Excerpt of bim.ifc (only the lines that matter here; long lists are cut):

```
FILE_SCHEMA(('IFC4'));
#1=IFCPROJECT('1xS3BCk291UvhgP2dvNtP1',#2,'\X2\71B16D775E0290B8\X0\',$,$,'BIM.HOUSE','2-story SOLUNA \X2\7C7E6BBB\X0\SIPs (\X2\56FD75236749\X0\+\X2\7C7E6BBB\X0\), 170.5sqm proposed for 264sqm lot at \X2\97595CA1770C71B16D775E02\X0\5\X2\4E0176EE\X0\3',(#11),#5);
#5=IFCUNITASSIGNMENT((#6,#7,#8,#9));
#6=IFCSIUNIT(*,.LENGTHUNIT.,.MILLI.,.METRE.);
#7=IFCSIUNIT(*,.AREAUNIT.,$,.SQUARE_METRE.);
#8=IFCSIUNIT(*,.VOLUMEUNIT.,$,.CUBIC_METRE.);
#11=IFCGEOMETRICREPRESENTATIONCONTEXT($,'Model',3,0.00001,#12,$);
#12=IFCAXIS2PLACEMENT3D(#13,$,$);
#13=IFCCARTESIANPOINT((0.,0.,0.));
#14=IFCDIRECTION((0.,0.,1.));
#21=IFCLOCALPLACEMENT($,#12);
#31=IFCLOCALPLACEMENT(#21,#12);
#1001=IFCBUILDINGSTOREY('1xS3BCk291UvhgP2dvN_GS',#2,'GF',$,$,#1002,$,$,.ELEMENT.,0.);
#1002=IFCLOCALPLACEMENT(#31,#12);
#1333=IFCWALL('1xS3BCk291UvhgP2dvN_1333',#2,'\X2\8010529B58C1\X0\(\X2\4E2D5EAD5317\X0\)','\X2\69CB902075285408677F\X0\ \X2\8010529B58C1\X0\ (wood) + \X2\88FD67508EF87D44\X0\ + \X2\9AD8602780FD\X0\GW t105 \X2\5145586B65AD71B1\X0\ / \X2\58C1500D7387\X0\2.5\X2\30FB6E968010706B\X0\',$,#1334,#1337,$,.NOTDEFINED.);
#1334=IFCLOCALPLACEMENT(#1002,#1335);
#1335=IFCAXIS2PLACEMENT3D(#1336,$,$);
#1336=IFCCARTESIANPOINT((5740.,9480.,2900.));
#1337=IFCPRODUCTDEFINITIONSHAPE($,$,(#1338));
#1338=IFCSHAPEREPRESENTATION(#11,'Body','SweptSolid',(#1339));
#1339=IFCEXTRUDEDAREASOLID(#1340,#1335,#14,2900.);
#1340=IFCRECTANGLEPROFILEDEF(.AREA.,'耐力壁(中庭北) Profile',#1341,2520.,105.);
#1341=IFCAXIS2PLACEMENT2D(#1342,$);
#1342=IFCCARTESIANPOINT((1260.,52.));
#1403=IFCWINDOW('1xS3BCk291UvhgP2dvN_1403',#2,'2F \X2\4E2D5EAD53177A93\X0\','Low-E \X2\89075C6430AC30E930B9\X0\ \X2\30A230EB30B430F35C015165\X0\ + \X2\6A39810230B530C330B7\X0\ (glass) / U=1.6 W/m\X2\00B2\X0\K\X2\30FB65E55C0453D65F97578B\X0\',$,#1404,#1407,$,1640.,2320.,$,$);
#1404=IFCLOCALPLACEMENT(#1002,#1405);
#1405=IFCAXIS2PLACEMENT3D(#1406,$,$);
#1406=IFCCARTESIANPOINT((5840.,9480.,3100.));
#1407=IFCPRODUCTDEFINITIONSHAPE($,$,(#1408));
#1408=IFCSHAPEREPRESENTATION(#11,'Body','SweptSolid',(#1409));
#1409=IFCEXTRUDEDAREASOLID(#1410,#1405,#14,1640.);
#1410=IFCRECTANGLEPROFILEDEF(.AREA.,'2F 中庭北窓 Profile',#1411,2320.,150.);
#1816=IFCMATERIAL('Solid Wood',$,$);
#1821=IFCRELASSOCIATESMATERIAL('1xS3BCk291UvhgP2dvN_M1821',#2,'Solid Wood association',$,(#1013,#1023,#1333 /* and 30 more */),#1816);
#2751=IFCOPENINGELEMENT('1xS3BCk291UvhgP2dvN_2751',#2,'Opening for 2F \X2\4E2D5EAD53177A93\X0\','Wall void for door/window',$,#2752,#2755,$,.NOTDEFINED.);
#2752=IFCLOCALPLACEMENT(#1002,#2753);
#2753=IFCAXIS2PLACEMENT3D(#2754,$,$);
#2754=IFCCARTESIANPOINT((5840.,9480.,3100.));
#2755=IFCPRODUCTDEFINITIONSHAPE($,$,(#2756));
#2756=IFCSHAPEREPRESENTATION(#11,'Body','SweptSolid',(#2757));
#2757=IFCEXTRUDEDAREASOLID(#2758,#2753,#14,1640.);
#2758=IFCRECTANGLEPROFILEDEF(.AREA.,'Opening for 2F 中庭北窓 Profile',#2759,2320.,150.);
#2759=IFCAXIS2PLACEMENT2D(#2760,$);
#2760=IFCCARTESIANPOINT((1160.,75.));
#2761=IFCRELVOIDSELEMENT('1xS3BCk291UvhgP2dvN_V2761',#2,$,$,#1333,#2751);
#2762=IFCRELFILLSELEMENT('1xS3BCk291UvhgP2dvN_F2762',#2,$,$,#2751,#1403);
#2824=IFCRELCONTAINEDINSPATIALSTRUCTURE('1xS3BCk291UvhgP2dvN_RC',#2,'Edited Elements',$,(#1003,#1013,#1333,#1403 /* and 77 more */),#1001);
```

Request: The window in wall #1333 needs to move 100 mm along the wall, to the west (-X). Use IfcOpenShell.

```python
import ifcopenshell
import ifcopenshell.api.geometry
import ifcopenshell.util.placement

model = ifcopenshell.open("bim.ifc")

window = model.by_guid("1xS3BCk291UvhgP2dvN_1403")
opening = window.FillsVoids[0].RelatingOpeningElement
wall = opening.VoidsElements[0].RelatingBuildingElement

wall_matrix = ifcopenshell.util.placement.get_local_placement(wall.ObjectPlacement)
shift = wall_matrix[:3, 0] * -100.0
before = ifcopenshell.util.placement.get_local_placement(window.ObjectPlacement)[:3, 3].copy()

# The window is not placed relative to its opening, so move both.
for product in (opening, window):
    matrix = ifcopenshell.util.placement.get_local_placement(product.ObjectPlacement)
    matrix[:3, 3] += shift
    ifcopenshell.api.geometry.edit_object_placement(model, product=product, matrix=matrix, is_si=False)

after = ifcopenshell.util.placement.get_local_placement(window.ObjectPlacement)[:3, 3]
print("window moved by", (after - before).round(3) + 0.0)

model.write("bim_v2.ifc")
```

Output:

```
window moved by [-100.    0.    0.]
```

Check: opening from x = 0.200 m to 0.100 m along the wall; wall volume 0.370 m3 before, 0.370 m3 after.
